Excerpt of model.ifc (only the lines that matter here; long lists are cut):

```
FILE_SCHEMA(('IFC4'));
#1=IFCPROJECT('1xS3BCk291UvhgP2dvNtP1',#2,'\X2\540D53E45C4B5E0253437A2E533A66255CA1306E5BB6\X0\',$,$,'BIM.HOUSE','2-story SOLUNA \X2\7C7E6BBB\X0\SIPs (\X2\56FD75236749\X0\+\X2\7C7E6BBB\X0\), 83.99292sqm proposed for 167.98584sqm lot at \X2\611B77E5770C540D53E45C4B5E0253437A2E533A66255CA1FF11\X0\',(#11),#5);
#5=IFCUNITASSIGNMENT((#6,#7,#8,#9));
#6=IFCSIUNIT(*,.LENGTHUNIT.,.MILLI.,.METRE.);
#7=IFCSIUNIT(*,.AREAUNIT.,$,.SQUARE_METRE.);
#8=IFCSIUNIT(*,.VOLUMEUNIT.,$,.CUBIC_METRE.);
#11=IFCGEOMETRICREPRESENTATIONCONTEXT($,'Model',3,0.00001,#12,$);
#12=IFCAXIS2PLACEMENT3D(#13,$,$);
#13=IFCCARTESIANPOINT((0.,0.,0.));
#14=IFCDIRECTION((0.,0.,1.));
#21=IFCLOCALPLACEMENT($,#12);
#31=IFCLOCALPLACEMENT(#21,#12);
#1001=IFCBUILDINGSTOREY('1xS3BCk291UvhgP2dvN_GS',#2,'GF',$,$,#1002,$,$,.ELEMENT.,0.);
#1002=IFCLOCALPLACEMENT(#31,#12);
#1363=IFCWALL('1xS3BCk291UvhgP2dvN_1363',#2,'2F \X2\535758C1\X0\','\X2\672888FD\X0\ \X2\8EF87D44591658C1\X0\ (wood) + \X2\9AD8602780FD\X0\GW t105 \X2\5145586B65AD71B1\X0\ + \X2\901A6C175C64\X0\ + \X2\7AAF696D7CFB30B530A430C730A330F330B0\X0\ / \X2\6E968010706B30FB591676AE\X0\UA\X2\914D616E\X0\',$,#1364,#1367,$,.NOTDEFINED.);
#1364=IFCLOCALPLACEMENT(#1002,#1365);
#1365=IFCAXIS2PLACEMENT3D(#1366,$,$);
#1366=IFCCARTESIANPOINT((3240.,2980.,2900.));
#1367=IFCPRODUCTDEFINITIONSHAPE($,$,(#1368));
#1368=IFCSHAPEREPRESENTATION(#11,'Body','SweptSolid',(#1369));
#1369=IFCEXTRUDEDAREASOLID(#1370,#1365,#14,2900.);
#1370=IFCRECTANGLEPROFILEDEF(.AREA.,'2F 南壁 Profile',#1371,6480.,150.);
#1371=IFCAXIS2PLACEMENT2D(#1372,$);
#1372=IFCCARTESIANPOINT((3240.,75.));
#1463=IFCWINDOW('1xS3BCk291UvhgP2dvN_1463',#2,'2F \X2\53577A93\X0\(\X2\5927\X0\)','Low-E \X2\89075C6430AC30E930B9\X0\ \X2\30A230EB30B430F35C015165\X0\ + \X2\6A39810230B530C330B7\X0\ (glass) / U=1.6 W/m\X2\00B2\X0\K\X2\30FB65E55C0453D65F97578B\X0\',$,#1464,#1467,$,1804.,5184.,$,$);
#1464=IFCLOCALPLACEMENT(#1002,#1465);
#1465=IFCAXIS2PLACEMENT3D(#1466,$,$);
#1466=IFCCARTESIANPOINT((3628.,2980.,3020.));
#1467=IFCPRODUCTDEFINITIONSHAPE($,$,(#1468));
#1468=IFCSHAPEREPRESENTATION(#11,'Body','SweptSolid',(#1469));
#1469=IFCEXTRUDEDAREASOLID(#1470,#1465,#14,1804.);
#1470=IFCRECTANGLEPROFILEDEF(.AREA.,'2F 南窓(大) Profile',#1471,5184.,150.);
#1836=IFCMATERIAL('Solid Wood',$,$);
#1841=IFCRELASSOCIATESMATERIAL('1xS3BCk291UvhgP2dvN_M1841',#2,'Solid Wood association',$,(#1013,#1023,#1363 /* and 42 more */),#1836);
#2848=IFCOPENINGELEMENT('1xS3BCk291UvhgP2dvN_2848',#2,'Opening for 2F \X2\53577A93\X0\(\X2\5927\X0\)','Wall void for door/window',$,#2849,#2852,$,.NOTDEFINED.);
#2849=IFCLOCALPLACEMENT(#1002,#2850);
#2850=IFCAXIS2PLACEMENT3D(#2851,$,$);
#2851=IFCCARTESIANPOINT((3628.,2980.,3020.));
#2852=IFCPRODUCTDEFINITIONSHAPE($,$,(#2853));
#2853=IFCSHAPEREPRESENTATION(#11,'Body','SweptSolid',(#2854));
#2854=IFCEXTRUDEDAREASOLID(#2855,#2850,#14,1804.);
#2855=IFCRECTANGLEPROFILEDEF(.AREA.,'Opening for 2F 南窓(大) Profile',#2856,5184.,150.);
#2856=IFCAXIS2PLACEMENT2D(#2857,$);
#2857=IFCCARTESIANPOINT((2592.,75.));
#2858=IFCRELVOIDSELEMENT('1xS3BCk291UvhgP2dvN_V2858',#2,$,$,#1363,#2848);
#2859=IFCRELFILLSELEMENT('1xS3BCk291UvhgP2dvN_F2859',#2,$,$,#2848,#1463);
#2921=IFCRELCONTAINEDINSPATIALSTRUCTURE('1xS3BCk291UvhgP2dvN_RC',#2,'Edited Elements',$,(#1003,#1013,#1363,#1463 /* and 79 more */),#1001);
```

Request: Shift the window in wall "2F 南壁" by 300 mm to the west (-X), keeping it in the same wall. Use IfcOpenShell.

```python
import ifcopenshell
import ifcopenshell.api.geometry
import ifcopenshell.util.placement
import ifcopenshell.util.unit

model = ifcopenshell.open("model.ifc")
unit_scale = ifcopenshell.util.unit.calculate_unit_scale(model)

window = model.by_guid("1xS3BCk291UvhgP2dvN_1463")
opening = window.FillsVoids[0].RelatingOpeningElement
wall = opening.VoidsElements[0].RelatingBuildingElement

wall_matrix = ifcopenshell.util.placement.get_local_placement(wall.ObjectPlacement)
shift = wall_matrix[:3, 0] * -0.3 / unit_scale
before = ifcopenshell.util.placement.get_local_placement(window.ObjectPlacement)[:3, 3].copy()

# The window is not placed relative to its opening, so move both.
for product in (opening, window):
    matrix = ifcopenshell.util.placement.get_local_placement(product.ObjectPlacement)
    matrix[:3, 3] += shift
    ifcopenshell.api.geometry.edit_object_placement(model, product=product, matrix=matrix, is_si=False)

after = ifcopenshell.util.placement.get_local_placement(window.ObjectPlacement)[:3, 3]
print("window moved by", (after - before).round(3) + 0.0)

model.write("model_edited.ifc")
```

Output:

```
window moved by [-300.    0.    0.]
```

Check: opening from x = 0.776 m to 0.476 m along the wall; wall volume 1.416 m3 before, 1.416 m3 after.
